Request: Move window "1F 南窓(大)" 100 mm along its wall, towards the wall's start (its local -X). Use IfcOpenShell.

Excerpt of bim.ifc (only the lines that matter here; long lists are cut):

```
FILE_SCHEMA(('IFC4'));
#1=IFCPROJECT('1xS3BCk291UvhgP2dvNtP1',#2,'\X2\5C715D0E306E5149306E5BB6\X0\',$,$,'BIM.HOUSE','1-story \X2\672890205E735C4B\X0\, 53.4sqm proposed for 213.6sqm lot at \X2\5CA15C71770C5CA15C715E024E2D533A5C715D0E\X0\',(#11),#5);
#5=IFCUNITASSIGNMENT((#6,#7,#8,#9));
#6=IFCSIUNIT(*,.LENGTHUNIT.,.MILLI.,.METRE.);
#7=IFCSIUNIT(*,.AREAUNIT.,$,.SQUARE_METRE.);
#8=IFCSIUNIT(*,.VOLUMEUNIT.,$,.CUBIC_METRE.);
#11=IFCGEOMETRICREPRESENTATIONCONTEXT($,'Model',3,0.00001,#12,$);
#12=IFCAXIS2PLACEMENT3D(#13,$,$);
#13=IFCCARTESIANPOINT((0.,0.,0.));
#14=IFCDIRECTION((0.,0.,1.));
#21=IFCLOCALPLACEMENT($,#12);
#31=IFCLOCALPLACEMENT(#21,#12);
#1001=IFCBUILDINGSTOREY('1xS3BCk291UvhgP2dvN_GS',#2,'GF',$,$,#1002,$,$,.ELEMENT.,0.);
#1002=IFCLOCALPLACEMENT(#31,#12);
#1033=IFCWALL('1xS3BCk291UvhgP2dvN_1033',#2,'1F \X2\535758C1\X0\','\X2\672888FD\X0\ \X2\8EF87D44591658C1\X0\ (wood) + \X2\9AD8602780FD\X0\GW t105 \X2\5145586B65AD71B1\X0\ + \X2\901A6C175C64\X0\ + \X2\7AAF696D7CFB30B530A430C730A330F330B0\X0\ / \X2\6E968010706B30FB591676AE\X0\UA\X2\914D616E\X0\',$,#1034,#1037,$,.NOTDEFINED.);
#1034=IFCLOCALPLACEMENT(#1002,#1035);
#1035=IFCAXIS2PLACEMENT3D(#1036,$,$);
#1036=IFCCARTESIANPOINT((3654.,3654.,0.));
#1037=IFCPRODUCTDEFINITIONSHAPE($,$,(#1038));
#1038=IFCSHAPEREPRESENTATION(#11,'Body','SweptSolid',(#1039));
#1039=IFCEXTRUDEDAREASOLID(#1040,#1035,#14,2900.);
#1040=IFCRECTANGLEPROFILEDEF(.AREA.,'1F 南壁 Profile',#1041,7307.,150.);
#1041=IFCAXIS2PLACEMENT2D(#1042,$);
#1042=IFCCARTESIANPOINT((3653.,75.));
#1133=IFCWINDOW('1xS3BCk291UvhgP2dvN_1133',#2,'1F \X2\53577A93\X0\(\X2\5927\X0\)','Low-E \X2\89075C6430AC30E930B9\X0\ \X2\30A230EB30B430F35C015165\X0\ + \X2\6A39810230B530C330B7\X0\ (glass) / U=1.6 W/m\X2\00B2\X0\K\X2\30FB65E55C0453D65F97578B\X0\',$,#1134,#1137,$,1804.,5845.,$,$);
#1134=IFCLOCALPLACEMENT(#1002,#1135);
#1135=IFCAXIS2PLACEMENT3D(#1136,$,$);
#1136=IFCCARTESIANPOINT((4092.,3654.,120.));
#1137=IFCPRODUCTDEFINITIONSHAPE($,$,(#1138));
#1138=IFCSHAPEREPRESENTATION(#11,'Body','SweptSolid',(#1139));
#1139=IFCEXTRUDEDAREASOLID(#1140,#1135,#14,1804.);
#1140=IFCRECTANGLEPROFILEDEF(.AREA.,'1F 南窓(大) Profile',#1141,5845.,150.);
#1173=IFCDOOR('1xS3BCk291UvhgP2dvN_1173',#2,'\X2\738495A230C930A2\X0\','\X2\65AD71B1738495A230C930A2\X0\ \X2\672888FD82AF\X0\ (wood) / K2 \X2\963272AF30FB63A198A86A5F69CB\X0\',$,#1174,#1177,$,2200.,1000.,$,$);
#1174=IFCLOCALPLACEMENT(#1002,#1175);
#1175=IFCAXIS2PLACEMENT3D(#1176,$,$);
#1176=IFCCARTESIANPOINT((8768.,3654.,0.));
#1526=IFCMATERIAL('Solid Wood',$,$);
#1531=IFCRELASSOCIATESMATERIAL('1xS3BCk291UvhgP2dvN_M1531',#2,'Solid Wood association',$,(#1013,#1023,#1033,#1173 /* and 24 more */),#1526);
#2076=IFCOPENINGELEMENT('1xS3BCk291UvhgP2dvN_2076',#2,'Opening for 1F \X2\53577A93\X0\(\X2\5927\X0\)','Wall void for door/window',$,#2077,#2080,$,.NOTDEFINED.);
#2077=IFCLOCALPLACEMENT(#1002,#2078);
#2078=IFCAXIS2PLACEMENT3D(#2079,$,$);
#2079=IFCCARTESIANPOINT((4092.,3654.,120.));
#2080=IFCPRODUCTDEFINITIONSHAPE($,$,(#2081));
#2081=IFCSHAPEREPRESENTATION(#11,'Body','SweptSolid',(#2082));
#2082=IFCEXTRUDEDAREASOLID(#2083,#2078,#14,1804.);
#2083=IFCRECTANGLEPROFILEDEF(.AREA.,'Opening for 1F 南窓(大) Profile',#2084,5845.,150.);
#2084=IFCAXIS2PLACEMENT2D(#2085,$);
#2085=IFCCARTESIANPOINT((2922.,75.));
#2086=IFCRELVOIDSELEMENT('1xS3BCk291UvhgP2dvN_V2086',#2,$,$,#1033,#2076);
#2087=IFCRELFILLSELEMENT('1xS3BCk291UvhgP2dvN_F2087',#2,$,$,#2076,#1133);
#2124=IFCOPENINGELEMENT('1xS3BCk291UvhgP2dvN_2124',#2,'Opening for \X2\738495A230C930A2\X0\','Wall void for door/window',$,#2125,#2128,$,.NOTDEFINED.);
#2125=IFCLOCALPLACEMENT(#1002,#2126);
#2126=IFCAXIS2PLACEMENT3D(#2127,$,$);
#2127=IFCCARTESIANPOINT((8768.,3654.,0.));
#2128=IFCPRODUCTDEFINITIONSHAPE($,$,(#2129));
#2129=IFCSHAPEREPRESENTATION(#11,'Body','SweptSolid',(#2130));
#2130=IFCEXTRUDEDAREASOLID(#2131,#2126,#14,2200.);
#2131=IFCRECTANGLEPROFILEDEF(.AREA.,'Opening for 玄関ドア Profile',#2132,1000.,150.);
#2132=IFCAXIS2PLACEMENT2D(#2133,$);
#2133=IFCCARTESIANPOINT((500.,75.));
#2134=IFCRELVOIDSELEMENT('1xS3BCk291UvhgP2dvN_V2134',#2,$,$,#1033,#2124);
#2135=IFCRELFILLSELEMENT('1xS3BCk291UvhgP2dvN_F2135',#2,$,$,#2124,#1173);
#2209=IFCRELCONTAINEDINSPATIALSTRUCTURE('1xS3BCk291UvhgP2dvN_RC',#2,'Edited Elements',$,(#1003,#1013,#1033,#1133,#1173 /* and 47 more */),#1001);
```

```python
import ifcopenshell
import ifcopenshell.api.geometry
import ifcopenshell.util.placement
import ifcopenshell.util.unit

model = ifcopenshell.open("bim.ifc")
unit_scale = ifcopenshell.util.unit.calculate_unit_scale(model)

window = model.by_guid("1xS3BCk291UvhgP2dvN_1133")
opening = window.FillsVoids[0].RelatingOpeningElement
wall = opening.VoidsElements[0].RelatingBuildingElement

wall_matrix = ifcopenshell.util.placement.get_local_placement(wall.ObjectPlacement)
shift = wall_matrix[:3, 0] * -0.1 / unit_scale
before = ifcopenshell.util.placement.get_local_placement(window.ObjectPlacement)[:3, 3].copy()

# The window is not placed relative to its opening, so move both.
for product in (opening, window):
    matrix = ifcopenshell.util.placement.get_local_placement(product.ObjectPlacement)
    matrix[:3, 3] += shift
    ifcopenshell.api.geometry.edit_object_placement(model, product=product, matrix=matrix, is_si=False)

after = ifcopenshell.util.placement.get_local_placement(window.ObjectPlacement)[:3, 3]
print("window moved by", (after - before).round(3) + 0.0)

model.write("bim-out.ifc")
```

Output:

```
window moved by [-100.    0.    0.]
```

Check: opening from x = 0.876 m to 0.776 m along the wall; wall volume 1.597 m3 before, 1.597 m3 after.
